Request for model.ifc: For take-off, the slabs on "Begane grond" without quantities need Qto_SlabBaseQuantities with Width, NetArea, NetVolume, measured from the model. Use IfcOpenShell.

First a look at what the model holds.

```python
import ifcopenshell
import ifcopenshell.util.element
import ifcopenshell.util.unit

model = ifcopenshell.open("model.ifc")
print(model.schema)
for unit_type in ("LENGTHUNIT", "AREAUNIT", "VOLUMEUNIT"):
    print(unit_type, ifcopenshell.util.unit.calculate_unit_scale(model, unit_type))
storey = next(s for s in model.by_type("IfcBuildingStorey") if s.Name == "Begane grond")
slabs = [e for e in ifcopenshell.util.element.get_decomposition(storey) if e.is_a("IfcSlab")]
for e in sorted(slabs, key=lambda e: e.id()):
    print(e.id(), e.is_a(), e.Name, list(ifcopenshell.util.element.get_psets(e, qtos_only=True)), sep=" | ")
```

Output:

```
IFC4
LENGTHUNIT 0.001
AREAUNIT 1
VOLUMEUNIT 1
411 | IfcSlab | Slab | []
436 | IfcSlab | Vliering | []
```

```python
import ifcopenshell
import ifcopenshell.api.pset
import ifcopenshell.geom
import ifcopenshell.util.element
import ifcopenshell.util.shape
import ifcopenshell.util.unit

model = ifcopenshell.open("model.ifc")
unit_scale = ifcopenshell.util.unit.calculate_unit_scale(model)
area_scale = ifcopenshell.util.unit.calculate_unit_scale(model, "AREAUNIT")
volume_scale = ifcopenshell.util.unit.calculate_unit_scale(model, "VOLUMEUNIT")
settings = ifcopenshell.geom.settings()

storey = next(s for s in model.by_type("IfcBuildingStorey") if s.Name == "Begane grond")
slabs = [e for e in ifcopenshell.util.element.get_decomposition(storey) if e.is_a("IfcSlab")]

for e in sorted(slabs, key=lambda e: e.id()):
    if ifcopenshell.util.element.get_psets(e, qtos_only=True, should_inherit=False):
        continue
    # Geometry comes back in metres, in the element's own axes.
    shape = ifcopenshell.geom.create_shape(settings, e)
    values = {
        "Width": ifcopenshell.util.shape.get_z(shape.geometry) / unit_scale,
        "NetArea": ifcopenshell.util.shape.get_footprint_area(shape.geometry) / area_scale,
        "NetVolume": ifcopenshell.util.shape.get_volume(shape.geometry) / volume_scale,
    }
    qto = ifcopenshell.api.pset.add_qto(model, product=e, name="Qto_SlabBaseQuantities")
    ifcopenshell.api.pset.edit_qto(model, qto=qto, properties=values)
    print(e.id(), {k: round(v, 3) for k, v in values.items()})

model.write("model_edited.ifc")
```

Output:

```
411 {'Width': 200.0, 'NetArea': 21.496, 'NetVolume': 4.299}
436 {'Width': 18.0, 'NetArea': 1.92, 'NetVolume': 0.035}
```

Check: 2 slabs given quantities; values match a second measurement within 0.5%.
